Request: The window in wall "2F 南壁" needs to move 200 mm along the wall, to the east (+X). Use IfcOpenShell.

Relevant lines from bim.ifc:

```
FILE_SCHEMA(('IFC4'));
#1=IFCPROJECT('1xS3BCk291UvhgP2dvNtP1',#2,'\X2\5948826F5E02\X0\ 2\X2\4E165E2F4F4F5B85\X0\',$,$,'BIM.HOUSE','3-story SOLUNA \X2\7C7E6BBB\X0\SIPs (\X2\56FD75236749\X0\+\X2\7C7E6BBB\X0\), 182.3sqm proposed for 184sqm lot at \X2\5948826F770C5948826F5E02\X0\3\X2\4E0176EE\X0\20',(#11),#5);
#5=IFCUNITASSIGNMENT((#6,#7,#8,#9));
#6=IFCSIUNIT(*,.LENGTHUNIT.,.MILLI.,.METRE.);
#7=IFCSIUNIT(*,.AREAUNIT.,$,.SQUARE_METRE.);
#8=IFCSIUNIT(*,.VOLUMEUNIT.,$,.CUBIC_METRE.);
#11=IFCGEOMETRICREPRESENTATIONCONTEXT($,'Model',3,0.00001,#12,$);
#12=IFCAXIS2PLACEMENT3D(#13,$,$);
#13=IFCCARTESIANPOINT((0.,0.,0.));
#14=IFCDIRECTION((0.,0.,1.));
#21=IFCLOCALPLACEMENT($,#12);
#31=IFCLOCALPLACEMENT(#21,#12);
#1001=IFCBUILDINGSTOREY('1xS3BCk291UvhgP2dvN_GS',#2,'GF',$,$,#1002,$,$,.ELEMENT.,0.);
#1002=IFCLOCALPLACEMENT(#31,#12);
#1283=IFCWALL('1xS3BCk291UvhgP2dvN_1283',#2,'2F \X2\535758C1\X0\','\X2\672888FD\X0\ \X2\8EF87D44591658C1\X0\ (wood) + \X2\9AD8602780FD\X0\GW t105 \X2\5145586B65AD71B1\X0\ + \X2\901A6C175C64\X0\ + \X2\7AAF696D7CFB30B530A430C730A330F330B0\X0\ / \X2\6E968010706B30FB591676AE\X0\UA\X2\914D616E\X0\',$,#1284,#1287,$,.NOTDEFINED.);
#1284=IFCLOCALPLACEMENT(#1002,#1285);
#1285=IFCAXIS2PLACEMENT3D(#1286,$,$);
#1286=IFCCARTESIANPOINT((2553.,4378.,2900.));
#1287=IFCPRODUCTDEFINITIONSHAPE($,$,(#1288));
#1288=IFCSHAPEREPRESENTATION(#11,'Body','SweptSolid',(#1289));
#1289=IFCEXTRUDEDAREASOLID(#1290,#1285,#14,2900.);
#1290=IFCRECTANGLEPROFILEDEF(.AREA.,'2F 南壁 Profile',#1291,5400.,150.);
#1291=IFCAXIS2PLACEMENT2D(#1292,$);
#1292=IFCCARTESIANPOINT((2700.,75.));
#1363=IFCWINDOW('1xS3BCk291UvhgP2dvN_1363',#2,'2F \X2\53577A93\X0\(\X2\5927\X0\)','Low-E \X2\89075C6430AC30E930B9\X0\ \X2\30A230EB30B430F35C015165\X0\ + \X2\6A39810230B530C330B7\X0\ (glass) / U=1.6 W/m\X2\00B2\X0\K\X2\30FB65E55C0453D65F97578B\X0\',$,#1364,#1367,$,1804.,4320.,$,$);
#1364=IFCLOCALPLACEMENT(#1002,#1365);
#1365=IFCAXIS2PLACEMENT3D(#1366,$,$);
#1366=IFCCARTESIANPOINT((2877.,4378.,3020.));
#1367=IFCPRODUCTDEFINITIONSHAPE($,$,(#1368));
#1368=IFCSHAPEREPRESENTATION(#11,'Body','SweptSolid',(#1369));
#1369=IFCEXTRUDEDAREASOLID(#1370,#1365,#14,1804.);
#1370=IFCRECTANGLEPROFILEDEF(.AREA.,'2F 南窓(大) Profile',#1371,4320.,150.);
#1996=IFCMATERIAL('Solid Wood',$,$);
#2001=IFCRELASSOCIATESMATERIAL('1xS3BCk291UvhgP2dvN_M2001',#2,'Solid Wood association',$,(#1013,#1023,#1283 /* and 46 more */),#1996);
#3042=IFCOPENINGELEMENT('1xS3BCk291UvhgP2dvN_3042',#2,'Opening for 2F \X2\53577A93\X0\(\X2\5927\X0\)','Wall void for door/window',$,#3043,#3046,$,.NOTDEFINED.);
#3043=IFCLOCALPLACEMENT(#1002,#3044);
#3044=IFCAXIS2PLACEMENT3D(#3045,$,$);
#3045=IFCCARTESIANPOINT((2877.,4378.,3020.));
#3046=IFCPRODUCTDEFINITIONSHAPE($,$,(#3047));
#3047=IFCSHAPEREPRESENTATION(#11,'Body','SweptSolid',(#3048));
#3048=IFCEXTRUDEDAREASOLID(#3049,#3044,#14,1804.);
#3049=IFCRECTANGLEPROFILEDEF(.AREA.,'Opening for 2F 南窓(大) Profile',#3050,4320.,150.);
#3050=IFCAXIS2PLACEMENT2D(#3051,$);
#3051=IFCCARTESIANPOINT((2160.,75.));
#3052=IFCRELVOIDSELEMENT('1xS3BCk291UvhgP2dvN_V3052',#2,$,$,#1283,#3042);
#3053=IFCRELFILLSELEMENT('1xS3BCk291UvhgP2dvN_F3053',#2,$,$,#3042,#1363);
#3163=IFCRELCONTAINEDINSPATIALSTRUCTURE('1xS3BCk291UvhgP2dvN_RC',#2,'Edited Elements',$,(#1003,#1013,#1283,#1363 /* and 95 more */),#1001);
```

```python
import ifcopenshell
import ifcopenshell.api.geometry
import ifcopenshell.util.placement
import ifcopenshell.util.unit

model = ifcopenshell.open("bim.ifc")
unit_scale = ifcopenshell.util.unit.calculate_unit_scale(model)

window = model.by_guid("1xS3BCk291UvhgP2dvN_1363")
opening = window.FillsVoids[0].RelatingOpeningElement
wall = opening.VoidsElements[0].RelatingBuildingElement

wall_matrix = ifcopenshell.util.placement.get_local_placement(wall.ObjectPlacement)
shift = wall_matrix[:3, 0] * 0.2 / unit_scale
before = ifcopenshell.util.placement.get_local_placement(window.ObjectPlacement)[:3, 3].copy()

# The window is not placed relative to its opening, so move both.
for product in (opening, window):
    matrix = ifcopenshell.util.placement.get_local_placement(product.ObjectPlacement)
    matrix[:3, 3] += shift
    ifcopenshell.api.geometry.edit_object_placement(model, product=product, matrix=matrix, is_si=False)

after = ifcopenshell.util.placement.get_local_placement(window.ObjectPlacement)[:3, 3]
print("window moved by", (after - before).round(3) + 0.0)

model.write("bim-out.ifc")
```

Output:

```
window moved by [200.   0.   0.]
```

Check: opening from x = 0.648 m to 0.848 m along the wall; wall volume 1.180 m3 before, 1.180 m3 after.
